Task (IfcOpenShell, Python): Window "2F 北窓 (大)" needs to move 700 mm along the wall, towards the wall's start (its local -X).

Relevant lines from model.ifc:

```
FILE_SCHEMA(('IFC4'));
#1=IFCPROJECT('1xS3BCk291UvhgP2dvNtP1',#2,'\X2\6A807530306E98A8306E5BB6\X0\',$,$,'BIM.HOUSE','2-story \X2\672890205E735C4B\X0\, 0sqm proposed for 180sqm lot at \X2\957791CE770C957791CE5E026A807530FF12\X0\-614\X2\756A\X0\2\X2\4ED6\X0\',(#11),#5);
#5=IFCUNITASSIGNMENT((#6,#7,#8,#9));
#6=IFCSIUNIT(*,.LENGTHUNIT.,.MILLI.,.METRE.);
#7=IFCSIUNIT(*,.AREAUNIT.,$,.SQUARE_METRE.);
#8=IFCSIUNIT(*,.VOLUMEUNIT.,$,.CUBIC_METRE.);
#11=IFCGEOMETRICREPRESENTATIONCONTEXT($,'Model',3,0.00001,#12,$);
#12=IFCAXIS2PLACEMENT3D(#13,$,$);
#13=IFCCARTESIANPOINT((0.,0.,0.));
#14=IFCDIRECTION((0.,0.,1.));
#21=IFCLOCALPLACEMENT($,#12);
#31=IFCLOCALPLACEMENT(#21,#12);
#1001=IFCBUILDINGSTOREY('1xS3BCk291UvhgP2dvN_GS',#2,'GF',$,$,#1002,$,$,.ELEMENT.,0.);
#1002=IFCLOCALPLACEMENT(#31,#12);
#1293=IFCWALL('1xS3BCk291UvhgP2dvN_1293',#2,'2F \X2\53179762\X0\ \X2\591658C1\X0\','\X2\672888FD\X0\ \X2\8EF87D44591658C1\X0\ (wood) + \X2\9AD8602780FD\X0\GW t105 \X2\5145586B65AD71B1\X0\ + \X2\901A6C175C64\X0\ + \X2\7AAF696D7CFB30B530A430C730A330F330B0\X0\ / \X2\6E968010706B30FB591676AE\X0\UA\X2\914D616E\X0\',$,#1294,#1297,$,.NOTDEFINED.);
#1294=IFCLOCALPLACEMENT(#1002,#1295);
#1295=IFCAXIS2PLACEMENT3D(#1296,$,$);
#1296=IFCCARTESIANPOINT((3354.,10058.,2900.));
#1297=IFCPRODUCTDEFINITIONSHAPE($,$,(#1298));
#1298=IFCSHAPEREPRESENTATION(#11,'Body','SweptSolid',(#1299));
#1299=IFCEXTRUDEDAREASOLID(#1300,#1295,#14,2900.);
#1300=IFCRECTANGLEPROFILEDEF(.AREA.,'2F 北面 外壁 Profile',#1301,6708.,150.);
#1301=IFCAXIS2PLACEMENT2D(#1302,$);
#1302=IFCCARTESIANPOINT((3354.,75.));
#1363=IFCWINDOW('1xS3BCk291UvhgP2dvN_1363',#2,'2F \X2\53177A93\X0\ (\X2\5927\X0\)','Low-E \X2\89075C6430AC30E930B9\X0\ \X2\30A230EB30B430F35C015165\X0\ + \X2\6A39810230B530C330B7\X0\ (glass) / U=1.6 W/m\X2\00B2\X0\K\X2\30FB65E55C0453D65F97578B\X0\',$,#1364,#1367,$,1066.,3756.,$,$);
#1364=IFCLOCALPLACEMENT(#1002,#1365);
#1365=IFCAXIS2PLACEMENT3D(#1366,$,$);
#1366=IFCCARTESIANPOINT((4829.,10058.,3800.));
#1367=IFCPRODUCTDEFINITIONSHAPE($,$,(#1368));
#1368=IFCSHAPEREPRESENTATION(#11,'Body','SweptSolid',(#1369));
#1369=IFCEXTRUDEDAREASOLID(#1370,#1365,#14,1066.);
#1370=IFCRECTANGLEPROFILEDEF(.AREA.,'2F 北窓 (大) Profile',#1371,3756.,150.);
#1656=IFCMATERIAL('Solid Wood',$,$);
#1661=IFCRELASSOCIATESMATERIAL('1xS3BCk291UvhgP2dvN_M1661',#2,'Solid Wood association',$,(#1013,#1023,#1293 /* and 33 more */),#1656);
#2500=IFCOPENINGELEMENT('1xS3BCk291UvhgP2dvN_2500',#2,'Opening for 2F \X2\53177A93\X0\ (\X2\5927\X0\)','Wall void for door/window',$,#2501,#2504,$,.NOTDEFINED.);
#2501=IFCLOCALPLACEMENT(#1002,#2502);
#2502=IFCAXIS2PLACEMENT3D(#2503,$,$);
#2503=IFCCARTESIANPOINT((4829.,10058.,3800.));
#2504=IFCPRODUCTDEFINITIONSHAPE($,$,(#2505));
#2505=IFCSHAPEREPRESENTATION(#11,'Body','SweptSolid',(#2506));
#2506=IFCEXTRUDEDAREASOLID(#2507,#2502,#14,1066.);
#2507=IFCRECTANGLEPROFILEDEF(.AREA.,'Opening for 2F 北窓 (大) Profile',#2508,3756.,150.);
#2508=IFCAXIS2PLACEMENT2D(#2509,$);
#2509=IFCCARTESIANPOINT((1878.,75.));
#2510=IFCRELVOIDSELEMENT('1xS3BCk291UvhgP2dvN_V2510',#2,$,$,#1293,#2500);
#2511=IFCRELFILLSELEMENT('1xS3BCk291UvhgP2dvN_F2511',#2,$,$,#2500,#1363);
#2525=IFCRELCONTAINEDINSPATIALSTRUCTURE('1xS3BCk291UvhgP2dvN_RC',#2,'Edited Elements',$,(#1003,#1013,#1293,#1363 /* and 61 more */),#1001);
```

```python
import ifcopenshell
import ifcopenshell.api.geometry
import ifcopenshell.util.placement
import ifcopenshell.util.unit

model = ifcopenshell.open("model.ifc")
unit_scale = ifcopenshell.util.unit.calculate_unit_scale(model)

window = model.by_guid("1xS3BCk291UvhgP2dvN_1363")
opening = window.FillsVoids[0].RelatingOpeningElement
wall = opening.VoidsElements[0].RelatingBuildingElement

wall_matrix = ifcopenshell.util.placement.get_local_placement(wall.ObjectPlacement)
shift = wall_matrix[:3, 0] * -0.7 / unit_scale
before = ifcopenshell.util.placement.get_local_placement(window.ObjectPlacement)[:3, 3].copy()

# The window is not placed relative to its opening, so move both.
for product in (opening, window):
    matrix = ifcopenshell.util.placement.get_local_placement(product.ObjectPlacement)
    matrix[:3, 3] += shift
    ifcopenshell.api.geometry.edit_object_placement(model, product=product, matrix=matrix, is_si=False)

after = ifcopenshell.util.placement.get_local_placement(window.ObjectPlacement)[:3, 3]
print("window moved by", (after - before).round(3) + 0.0)

model.write("model_v2.ifc")
```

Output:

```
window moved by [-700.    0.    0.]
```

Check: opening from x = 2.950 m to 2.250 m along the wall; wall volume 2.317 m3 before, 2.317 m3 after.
